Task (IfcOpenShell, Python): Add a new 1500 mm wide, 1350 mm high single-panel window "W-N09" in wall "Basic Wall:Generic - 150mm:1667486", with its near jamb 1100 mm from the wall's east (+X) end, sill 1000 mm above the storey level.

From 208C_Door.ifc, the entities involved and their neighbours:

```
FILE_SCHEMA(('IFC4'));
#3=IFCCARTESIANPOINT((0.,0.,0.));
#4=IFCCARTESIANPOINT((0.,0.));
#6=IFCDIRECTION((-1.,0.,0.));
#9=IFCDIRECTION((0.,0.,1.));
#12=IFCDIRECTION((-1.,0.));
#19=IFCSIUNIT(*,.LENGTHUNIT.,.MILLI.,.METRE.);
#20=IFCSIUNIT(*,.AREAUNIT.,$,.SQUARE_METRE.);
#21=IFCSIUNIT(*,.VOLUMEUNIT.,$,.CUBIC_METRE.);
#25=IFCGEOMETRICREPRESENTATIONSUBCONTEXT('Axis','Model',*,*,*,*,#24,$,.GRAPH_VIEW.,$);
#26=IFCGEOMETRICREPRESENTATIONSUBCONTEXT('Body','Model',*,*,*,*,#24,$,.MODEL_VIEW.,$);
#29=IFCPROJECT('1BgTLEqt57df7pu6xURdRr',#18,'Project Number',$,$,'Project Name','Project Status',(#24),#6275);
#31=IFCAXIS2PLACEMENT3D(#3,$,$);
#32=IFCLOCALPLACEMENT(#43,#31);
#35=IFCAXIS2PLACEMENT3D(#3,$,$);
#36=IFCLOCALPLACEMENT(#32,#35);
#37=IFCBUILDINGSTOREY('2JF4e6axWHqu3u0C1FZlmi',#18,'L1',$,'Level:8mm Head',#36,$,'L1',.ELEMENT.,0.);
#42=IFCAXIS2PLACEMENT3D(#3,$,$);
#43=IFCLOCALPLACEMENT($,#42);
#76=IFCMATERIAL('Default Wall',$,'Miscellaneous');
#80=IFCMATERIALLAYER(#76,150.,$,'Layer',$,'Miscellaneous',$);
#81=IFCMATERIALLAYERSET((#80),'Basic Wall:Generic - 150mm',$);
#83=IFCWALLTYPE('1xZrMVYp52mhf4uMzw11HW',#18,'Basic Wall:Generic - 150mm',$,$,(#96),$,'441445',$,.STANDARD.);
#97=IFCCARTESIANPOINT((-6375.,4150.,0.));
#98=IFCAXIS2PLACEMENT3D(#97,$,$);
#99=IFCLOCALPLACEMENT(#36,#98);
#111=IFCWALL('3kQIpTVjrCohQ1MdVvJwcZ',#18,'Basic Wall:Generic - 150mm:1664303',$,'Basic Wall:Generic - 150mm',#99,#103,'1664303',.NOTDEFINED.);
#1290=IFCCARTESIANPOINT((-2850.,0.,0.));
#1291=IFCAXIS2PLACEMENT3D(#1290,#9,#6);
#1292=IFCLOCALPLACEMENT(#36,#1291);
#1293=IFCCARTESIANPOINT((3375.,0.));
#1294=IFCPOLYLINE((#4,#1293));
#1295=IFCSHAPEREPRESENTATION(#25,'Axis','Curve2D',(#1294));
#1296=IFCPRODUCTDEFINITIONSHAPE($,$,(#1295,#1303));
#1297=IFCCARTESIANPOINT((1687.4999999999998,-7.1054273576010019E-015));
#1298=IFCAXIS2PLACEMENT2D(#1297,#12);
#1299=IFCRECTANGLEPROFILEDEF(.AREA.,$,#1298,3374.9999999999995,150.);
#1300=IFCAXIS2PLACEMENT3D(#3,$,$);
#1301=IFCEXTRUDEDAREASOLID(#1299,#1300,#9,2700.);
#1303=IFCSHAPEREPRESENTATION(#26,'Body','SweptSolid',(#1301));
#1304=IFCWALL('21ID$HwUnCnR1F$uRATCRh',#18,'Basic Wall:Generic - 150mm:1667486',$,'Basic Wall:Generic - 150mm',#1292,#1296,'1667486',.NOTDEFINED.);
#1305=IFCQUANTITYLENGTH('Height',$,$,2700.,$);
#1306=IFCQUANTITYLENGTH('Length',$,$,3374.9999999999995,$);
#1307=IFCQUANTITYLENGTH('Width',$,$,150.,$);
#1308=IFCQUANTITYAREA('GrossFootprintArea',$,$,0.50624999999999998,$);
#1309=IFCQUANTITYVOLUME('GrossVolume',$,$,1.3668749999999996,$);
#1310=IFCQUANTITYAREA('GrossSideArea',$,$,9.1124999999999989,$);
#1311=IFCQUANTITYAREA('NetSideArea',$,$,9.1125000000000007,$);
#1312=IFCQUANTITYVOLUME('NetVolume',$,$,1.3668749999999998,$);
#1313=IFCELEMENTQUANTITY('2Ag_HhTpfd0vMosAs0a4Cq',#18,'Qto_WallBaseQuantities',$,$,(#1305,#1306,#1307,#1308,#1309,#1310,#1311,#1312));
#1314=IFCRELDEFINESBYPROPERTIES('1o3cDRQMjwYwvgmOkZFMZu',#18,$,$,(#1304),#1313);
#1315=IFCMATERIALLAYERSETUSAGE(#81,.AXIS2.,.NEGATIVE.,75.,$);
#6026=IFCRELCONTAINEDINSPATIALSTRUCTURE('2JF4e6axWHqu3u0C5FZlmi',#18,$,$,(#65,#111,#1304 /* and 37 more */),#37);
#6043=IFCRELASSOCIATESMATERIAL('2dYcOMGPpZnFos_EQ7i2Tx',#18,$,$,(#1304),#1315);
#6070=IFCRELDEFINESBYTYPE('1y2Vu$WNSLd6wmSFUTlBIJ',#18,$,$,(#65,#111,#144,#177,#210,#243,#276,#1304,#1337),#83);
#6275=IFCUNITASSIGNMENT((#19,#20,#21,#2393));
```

```python
import numpy as np
import ifcopenshell
import ifcopenshell.api.feature
import ifcopenshell.api.geometry
import ifcopenshell.api.pset
import ifcopenshell.api.root
import ifcopenshell.api.spatial
import ifcopenshell.geom
import ifcopenshell.util.element
import ifcopenshell.util.placement
import ifcopenshell.util.representation
import ifcopenshell.util.shape
import ifcopenshell.util.unit

model = ifcopenshell.open("208C_Door.ifc")
unit_scale = ifcopenshell.util.unit.calculate_unit_scale(model)
area_scale = ifcopenshell.util.unit.calculate_unit_scale(model, "AREAUNIT")
volume_scale = ifcopenshell.util.unit.calculate_unit_scale(model, "VOLUMEUNIT")
settings = ifcopenshell.geom.settings()


def volume(element):
    """Net volume in cubic metres, openings subtracted."""
    shape = ifcopenshell.geom.create_shape(settings, element)
    return ifcopenshell.util.shape.get_volume(shape.geometry)


wall = model.by_guid("21ID$HwUnCnR1F$uRATCRh")
storey = ifcopenshell.util.element.get_container(wall, ifc_class="IfcBuildingStorey")
context = ifcopenshell.util.representation.get_context(model, "Model", "Body", "MODEL_VIEW")
before = volume(wall)

width, height, from_end, sill = 1.5, 1.35, 1.1, 1  # metres

# The wall runs along its own X axis, and the end named is its -X end.
wall_shape = ifcopenshell.geom.create_shape(settings, wall)
x, y, z = ifcopenshell.util.shape.get_vertices(wall_shape.geometry).T
start = x.min() + from_end
face, thickness = float(y.min()), float(y.max() - y.min())
wall_matrix = ifcopenshell.util.placement.get_local_placement(wall.ObjectPlacement)
level = ifcopenshell.util.placement.get_local_placement(storey.ObjectPlacement)[2, 3]


def in_wall(x, y):
    """Placement at x, y metres in the wall's axes, at sill height."""
    matrix = wall_matrix.copy()
    matrix[:, 3] = wall_matrix @ np.array([x / unit_scale, y / unit_scale, 0.0, 1.0])
    matrix[2, 3] = level + sill / unit_scale
    return matrix


# Opening: a box that overshoots both wall faces by 50 mm.
opening = ifcopenshell.api.root.create_entity(model, ifc_class="IfcOpeningElement", predefined_type="OPENING")
box = ifcopenshell.api.geometry.add_wall_representation(
    model, context=context, length=width, height=height, thickness=thickness + 0.1
)
ifcopenshell.api.geometry.assign_representation(model, product=opening, representation=box)
ifcopenshell.api.geometry.edit_object_placement(model, product=opening, matrix=in_wall(start, face - 0.05), is_si=False)
ifcopenshell.api.feature.add_feature(model, feature=opening, element=wall)

window = ifcopenshell.api.root.create_entity(model, ifc_class="IfcWindow", name="W-N09", predefined_type="WINDOW")
window.OverallWidth, window.OverallHeight = width / unit_scale, height / unit_scale
window.PartitioningType = "SINGLE_PANEL"
body = ifcopenshell.api.geometry.add_window_representation(
    model,
    context=context,
    overall_width=window.OverallWidth,
    overall_height=window.OverallHeight,
    partition_type="SINGLE_PANEL",
)
ifcopenshell.api.geometry.assign_representation(model, product=window, representation=body)
ifcopenshell.api.spatial.assign_container(model, products=[window], relating_structure=storey)
ifcopenshell.api.feature.add_filling(model, opening=opening, element=window)

# Centre the window in the wall's thickness.
ifcopenshell.api.geometry.edit_object_placement(model, product=window, matrix=in_wall(start, face), is_si=False)
window_shape = ifcopenshell.geom.create_shape(settings, window)
depth = ifcopenshell.util.shape.get_vertices(window_shape.geometry)[:, 1]
offset = face + thickness / 2 - (depth.min() + depth.max()) / 2
ifcopenshell.api.geometry.edit_object_placement(model, product=window, matrix=in_wall(start, offset), is_si=False)

after = volume(wall)

# Update the wall's stored quantities.
qto = model.by_id(ifcopenshell.util.element.get_pset(wall, "Qto_WallBaseQuantities", should_inherit=False)["id"])
ifcopenshell.api.pset.edit_qto(model, qto=qto, properties={
    "NetSideArea": after / thickness / area_scale,
    "NetVolume": after / volume_scale,
})

print(f"wall volume {before:.3f} -> {after:.3f} m3")

model.write("208C_Door_rev.ifc")
```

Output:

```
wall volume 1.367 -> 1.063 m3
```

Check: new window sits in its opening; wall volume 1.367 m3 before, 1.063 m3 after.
